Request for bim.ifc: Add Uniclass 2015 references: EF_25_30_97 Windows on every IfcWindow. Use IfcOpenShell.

First a look at what the model holds.

```python
import ifcopenshell

model = ifcopenshell.open("bim.ifc")
print(model.schema)
print("classifications:", [c.Name for c in model.by_type("IfcClassification")])
for ifc_class in ("IfcDoor", "IfcRoof", "IfcStair", "IfcWall", "IfcWindow"):
    print(ifc_class, len(model.by_type(ifc_class)))
```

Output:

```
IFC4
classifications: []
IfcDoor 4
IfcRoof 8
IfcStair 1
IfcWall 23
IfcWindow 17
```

```python
import ifcopenshell
import ifcopenshell.api.classification

model = ifcopenshell.open("bim.ifc")

system = ifcopenshell.api.classification.add_classification(model, classification="Uniclass 2015")

codes = {
    "IfcWindow": ("EF_25_30_97", "Windows"),
}
for ifc_class, (code, name) in codes.items():
    products = model.by_type(ifc_class)
    ifcopenshell.api.classification.add_reference(
        model, products=products, classification=system, identification=code, name=name
    )
    print(code, len(products))

model.write("bim_rev.ifc")
```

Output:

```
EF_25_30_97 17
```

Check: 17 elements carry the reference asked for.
